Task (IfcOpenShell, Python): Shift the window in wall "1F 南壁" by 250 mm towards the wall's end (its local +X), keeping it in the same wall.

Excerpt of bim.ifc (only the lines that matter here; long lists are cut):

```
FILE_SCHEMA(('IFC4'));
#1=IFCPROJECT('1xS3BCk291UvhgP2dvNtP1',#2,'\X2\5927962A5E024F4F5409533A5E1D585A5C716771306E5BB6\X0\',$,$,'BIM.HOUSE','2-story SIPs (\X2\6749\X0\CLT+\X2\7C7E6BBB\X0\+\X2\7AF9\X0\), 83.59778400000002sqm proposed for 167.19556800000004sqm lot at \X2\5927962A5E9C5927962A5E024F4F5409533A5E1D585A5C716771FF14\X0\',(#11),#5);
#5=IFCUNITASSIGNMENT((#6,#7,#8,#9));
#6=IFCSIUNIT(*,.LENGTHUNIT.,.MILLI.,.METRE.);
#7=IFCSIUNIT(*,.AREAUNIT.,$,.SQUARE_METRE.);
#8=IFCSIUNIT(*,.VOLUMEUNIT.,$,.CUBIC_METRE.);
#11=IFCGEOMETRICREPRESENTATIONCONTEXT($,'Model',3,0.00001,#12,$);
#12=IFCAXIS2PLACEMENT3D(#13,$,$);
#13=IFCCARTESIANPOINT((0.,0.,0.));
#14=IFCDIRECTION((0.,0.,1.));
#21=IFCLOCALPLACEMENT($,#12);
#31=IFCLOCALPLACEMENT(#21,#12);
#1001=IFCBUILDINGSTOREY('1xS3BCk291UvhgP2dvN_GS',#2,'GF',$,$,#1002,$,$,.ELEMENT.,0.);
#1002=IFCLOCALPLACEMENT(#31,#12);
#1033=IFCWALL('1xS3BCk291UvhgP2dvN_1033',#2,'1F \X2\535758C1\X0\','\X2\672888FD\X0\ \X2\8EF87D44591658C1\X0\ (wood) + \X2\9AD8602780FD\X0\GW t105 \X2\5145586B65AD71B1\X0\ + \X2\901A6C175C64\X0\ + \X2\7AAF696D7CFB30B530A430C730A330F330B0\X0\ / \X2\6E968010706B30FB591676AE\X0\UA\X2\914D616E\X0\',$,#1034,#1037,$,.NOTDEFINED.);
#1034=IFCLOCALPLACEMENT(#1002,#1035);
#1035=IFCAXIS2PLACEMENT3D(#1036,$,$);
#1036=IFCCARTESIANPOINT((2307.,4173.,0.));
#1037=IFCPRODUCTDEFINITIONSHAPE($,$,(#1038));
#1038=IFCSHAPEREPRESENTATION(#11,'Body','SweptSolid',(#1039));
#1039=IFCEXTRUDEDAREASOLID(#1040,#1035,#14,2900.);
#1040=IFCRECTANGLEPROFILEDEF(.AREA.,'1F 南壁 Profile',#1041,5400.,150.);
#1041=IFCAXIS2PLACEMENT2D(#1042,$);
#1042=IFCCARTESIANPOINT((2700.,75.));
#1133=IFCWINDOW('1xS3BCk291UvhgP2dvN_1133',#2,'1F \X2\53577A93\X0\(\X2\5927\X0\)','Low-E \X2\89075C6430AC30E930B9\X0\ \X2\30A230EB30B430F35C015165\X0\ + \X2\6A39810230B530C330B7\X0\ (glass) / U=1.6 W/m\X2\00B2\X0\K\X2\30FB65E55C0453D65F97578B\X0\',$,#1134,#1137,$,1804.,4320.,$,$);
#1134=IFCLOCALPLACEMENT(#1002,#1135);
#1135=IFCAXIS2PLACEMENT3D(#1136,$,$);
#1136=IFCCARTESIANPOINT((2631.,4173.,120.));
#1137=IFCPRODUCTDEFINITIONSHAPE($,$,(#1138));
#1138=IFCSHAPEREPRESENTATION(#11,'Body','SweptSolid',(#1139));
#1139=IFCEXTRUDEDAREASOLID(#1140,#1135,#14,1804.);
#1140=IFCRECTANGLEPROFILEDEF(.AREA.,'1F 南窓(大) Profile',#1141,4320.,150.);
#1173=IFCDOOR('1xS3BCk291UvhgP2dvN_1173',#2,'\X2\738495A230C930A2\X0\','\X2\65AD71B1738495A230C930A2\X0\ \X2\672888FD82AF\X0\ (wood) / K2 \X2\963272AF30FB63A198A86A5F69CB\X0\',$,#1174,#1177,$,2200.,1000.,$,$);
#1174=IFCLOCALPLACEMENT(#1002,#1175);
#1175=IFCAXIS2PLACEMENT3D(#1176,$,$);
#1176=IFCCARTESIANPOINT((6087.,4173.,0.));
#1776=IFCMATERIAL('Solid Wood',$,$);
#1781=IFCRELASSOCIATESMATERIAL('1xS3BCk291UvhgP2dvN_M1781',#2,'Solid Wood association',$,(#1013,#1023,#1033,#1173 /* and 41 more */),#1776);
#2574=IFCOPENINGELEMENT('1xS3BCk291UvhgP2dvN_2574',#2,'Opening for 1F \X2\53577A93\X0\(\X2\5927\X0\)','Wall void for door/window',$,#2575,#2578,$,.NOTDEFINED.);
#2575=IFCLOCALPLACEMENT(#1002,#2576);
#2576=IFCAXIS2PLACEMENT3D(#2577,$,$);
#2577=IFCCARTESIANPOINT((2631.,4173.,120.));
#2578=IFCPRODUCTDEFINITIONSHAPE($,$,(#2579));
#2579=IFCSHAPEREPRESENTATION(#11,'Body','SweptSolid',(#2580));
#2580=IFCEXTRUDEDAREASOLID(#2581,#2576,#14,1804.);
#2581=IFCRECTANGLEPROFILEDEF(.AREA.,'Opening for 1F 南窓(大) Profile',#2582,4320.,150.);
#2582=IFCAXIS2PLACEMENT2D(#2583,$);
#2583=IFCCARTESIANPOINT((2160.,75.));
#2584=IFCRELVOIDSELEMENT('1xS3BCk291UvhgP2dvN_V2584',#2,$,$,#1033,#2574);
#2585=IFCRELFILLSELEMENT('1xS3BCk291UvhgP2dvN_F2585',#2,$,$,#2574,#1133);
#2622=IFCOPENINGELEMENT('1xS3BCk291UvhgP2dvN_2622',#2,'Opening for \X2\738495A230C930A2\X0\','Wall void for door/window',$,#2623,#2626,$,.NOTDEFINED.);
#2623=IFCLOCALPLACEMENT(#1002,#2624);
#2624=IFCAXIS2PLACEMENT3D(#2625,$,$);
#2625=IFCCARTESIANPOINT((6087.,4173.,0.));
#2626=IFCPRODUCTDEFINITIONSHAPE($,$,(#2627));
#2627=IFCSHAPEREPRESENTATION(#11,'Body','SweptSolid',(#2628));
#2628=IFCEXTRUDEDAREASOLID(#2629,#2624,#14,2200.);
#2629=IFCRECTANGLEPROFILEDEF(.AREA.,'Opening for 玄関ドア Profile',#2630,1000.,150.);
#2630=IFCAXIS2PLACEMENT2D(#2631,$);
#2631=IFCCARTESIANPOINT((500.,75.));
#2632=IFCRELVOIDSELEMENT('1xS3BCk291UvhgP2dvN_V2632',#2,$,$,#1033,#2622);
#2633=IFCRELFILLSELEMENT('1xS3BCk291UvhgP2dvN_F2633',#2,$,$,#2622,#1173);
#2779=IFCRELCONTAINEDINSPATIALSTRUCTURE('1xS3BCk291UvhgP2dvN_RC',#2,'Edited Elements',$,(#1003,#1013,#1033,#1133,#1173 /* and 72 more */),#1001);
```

```python
import ifcopenshell
import ifcopenshell.api.geometry
import ifcopenshell.util.placement
import ifcopenshell.util.unit

model = ifcopenshell.open("bim.ifc")
unit_scale = ifcopenshell.util.unit.calculate_unit_scale(model)

window = model.by_id(1133)
opening = window.FillsVoids[0].RelatingOpeningElement
wall = opening.VoidsElements[0].RelatingBuildingElement

wall_matrix = ifcopenshell.util.placement.get_local_placement(wall.ObjectPlacement)
shift = wall_matrix[:3, 0] * 0.25 / unit_scale
before = ifcopenshell.util.placement.get_local_placement(window.ObjectPlacement)[:3, 3].copy()

# The window is not placed relative to its opening, so move both.
for product in (opening, window):
    matrix = ifcopenshell.util.placement.get_local_placement(product.ObjectPlacement)
    matrix[:3, 3] += shift
    ifcopenshell.api.geometry.edit_object_placement(model, product=product, matrix=matrix, is_si=False)

after = ifcopenshell.util.placement.get_local_placement(window.ObjectPlacement)[:3, 3]
print("window moved by", (after - before).round(3) + 0.0)

model.write("bim_rev.ifc")
```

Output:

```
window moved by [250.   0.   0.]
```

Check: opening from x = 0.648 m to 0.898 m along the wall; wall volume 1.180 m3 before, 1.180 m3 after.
